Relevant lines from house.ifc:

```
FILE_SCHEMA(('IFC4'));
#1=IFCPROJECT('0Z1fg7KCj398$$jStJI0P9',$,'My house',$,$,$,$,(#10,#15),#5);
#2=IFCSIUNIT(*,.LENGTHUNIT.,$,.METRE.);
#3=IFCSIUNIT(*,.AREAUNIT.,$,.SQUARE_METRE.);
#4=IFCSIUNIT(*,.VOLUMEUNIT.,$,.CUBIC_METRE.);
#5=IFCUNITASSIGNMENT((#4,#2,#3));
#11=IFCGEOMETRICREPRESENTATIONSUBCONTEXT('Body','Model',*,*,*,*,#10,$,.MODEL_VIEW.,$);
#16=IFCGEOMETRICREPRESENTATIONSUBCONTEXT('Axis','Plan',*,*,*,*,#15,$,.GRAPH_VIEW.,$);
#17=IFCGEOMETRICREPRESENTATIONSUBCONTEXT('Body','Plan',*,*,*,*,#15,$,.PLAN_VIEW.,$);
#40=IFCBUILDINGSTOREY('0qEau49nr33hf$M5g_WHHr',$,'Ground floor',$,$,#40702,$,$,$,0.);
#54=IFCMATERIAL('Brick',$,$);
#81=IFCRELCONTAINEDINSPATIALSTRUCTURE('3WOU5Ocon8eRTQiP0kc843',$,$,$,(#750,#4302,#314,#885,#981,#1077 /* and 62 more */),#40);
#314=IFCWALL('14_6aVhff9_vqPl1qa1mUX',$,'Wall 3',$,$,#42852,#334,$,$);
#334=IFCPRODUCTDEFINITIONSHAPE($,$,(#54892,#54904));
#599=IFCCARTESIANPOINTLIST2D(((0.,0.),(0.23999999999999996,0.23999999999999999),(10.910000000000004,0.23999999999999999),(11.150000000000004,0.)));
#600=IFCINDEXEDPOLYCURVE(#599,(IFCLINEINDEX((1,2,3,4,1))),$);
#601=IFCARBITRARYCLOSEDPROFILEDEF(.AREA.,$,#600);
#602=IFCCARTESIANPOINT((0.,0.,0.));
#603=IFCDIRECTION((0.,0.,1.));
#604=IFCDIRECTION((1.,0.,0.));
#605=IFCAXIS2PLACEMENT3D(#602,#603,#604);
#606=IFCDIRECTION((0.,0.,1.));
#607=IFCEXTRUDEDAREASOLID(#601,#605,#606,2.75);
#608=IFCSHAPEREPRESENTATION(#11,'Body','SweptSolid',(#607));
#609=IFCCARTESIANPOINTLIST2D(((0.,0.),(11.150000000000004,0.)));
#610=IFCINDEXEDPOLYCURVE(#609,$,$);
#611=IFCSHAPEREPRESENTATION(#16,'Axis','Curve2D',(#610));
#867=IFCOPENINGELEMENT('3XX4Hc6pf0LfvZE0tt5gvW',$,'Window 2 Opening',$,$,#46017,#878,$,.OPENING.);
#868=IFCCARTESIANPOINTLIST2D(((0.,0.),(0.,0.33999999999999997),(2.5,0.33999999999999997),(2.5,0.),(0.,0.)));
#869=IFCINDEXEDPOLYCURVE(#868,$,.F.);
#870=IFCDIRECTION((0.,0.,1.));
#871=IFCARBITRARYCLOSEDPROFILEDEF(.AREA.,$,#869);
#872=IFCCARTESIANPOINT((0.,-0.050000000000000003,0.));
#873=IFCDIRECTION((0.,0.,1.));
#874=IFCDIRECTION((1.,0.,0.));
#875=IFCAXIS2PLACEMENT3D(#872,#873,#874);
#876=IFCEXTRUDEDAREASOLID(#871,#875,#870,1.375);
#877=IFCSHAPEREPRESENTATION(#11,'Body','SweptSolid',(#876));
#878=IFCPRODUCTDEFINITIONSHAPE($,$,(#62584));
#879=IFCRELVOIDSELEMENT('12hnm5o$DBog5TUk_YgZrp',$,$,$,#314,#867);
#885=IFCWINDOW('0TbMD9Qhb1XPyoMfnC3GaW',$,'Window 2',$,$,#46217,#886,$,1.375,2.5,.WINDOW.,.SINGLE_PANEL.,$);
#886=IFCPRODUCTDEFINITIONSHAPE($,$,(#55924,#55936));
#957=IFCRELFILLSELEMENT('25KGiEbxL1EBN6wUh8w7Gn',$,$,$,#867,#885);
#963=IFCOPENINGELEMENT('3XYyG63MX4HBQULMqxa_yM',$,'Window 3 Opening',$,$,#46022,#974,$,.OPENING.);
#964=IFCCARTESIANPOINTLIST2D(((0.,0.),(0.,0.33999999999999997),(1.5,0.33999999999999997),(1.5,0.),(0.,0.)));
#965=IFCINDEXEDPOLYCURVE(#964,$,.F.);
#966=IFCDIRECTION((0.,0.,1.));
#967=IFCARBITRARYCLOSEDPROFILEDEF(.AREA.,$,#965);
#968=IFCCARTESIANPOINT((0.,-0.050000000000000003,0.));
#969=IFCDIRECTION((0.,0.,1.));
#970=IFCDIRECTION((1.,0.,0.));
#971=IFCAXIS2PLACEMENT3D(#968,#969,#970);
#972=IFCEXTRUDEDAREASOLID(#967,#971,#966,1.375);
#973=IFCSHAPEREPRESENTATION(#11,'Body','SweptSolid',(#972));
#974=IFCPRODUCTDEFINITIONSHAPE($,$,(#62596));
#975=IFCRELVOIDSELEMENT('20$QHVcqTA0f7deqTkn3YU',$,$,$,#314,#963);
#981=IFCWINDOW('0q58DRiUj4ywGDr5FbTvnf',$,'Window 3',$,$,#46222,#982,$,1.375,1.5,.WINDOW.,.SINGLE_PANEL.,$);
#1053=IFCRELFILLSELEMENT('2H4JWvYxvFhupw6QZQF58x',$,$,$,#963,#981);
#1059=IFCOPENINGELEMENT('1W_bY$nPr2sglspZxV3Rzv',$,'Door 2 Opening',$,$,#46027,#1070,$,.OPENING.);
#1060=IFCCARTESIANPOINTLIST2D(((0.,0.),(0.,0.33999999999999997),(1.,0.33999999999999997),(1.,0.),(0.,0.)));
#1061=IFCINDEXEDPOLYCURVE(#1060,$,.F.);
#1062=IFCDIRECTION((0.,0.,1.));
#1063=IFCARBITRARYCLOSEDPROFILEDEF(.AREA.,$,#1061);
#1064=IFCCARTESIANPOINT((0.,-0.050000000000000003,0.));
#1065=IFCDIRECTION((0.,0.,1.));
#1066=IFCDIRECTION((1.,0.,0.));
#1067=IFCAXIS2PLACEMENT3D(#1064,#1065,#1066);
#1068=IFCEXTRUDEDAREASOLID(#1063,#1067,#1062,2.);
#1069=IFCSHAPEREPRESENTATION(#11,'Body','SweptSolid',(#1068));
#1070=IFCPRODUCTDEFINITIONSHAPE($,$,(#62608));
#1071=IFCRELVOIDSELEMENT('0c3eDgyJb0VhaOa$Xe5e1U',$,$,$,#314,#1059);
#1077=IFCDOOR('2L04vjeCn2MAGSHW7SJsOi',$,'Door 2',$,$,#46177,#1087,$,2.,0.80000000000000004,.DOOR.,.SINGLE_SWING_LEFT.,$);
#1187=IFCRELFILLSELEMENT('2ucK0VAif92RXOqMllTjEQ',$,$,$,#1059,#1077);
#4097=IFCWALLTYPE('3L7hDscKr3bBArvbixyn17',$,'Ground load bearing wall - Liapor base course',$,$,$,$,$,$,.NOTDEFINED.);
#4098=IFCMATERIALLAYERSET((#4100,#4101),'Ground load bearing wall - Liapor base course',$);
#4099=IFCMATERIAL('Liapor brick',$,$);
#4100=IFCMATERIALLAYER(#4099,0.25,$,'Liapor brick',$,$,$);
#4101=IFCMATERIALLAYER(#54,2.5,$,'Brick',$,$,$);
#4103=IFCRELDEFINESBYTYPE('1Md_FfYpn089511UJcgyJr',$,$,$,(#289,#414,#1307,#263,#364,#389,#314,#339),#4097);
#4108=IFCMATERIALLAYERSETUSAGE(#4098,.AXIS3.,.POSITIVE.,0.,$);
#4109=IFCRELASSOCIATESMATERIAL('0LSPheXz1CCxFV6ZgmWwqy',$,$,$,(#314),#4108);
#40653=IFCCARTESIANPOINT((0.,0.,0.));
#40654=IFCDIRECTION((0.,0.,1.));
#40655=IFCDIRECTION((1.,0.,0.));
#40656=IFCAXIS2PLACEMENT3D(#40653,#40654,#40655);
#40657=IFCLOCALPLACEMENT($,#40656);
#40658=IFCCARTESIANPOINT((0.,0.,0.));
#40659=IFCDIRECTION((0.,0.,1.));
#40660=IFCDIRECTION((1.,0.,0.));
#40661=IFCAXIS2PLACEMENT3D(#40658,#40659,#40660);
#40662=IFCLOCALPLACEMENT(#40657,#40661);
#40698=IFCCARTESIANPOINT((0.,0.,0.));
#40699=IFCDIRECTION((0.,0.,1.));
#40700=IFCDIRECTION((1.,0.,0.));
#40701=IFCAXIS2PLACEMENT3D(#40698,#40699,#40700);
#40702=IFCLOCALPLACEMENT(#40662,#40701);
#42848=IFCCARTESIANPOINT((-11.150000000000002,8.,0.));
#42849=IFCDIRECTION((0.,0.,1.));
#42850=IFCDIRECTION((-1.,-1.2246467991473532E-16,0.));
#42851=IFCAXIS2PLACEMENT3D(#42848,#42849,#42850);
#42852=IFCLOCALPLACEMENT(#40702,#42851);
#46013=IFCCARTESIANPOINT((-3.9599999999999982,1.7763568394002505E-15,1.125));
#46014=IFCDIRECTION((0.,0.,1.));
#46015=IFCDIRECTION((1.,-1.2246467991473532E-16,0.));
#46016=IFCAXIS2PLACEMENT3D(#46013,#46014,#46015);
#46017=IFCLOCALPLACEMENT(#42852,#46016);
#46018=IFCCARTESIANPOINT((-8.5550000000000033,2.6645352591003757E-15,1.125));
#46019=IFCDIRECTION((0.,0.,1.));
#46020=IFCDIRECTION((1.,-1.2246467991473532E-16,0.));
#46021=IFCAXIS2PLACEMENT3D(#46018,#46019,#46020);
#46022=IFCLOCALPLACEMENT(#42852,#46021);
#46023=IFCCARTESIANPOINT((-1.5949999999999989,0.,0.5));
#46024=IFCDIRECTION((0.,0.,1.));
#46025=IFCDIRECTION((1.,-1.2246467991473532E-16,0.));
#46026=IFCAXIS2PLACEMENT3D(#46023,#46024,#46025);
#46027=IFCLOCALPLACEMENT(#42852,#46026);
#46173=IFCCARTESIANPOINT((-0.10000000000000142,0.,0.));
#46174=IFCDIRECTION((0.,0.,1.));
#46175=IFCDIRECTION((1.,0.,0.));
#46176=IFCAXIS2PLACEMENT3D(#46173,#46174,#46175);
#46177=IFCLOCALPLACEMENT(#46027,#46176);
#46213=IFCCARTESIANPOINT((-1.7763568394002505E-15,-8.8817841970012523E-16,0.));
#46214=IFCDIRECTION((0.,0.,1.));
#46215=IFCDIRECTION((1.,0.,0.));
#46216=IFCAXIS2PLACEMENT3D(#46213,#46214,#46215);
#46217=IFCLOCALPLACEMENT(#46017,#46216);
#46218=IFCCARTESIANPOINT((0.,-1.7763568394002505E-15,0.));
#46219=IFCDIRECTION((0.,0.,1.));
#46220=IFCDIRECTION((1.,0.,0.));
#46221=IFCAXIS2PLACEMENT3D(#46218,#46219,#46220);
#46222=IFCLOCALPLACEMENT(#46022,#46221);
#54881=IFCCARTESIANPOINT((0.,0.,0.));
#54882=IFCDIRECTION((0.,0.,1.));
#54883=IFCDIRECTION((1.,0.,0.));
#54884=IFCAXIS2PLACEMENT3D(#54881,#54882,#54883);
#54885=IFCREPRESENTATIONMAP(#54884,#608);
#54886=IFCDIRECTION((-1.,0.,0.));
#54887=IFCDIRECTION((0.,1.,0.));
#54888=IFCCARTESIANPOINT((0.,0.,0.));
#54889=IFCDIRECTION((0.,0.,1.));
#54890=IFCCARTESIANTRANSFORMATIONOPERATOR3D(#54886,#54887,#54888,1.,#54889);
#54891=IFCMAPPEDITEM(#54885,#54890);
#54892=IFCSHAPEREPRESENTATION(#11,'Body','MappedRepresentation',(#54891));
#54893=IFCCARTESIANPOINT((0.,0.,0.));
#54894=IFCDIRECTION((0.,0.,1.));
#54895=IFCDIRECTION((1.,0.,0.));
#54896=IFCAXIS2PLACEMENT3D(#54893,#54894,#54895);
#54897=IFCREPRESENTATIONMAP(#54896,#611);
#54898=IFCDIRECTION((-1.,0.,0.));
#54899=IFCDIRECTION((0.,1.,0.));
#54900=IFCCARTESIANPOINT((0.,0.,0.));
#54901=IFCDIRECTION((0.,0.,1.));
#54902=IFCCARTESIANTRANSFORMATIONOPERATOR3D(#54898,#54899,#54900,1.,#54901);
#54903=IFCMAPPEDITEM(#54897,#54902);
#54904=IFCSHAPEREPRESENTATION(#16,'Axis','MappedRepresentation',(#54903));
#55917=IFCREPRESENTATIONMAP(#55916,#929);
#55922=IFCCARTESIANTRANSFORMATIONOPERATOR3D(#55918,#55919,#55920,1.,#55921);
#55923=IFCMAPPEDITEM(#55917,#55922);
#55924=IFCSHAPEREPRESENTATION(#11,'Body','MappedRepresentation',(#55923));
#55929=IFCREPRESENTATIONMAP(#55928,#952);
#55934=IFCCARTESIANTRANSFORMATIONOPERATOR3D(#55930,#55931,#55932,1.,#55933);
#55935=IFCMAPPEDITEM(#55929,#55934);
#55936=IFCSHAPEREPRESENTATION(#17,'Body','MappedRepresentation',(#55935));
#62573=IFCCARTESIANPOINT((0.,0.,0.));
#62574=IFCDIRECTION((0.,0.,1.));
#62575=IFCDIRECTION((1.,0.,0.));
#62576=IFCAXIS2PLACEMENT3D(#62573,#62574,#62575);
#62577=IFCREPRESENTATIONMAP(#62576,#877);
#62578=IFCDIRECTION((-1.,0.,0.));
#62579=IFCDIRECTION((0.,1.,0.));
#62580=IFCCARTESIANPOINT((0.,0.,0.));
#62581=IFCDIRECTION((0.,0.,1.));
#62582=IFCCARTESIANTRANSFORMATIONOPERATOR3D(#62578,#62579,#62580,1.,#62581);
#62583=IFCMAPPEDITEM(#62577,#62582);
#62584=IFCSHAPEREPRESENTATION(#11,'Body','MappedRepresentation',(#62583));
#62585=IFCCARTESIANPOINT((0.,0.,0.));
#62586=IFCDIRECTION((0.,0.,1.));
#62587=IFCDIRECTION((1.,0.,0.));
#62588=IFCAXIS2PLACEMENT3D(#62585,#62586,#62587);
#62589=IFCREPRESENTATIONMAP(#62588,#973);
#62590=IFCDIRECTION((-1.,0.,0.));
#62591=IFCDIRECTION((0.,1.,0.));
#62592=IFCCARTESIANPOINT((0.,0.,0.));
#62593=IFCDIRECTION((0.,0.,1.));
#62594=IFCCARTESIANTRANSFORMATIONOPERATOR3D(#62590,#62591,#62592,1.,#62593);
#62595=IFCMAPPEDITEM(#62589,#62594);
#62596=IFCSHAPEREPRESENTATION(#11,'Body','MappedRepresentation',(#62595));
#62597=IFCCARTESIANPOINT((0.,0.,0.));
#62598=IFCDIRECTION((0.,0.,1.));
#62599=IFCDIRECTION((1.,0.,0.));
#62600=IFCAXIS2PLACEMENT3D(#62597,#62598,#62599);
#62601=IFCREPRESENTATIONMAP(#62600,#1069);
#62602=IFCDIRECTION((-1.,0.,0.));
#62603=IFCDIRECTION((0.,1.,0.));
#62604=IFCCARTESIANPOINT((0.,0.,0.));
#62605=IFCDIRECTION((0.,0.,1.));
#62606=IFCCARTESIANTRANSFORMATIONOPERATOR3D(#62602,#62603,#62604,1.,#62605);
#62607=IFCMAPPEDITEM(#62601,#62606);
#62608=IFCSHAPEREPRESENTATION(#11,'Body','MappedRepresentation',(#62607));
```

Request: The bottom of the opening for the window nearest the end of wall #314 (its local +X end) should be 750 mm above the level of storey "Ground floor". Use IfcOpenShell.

```python
import numpy as np
import ifcopenshell
import ifcopenshell.api.geometry
import ifcopenshell.geom
import ifcopenshell.util.element
import ifcopenshell.util.placement
import ifcopenshell.util.shape
import ifcopenshell.util.unit

model = ifcopenshell.open("house.ifc")
unit_scale = ifcopenshell.util.unit.calculate_unit_scale(model)

window = model.by_guid("0TbMD9Qhb1XPyoMfnC3GaW")
opening = window.FillsVoids[0].RelatingOpeningElement
storey = ifcopenshell.util.element.get_container(window, ifc_class="IfcBuildingStorey")
level = ifcopenshell.util.placement.get_local_placement(storey.ObjectPlacement)[2, 3]

# The opening's origin need not be at the sill, so measure its lowest point.
shape = ifcopenshell.geom.create_shape(ifcopenshell.geom.settings(), opening)
bottom = ifcopenshell.util.shape.get_shape_bottom_elevation(shape, shape.geometry) / unit_scale
dz = level + 0.75 - bottom

shift = np.array([0.0, 0.0, dz])
# The window is placed relative to its opening, so it follows when the opening moves.
matrix = ifcopenshell.util.placement.get_local_placement(opening.ObjectPlacement)
matrix[:3, 3] += shift
ifcopenshell.api.geometry.edit_object_placement(
    model, product=opening, matrix=matrix, is_si=False, should_transform_children=True
)

print(f"moved by {dz * unit_scale:+.3f} m")

model.write("house_v2.ifc")
```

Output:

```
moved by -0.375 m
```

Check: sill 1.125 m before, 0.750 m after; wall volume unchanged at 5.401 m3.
